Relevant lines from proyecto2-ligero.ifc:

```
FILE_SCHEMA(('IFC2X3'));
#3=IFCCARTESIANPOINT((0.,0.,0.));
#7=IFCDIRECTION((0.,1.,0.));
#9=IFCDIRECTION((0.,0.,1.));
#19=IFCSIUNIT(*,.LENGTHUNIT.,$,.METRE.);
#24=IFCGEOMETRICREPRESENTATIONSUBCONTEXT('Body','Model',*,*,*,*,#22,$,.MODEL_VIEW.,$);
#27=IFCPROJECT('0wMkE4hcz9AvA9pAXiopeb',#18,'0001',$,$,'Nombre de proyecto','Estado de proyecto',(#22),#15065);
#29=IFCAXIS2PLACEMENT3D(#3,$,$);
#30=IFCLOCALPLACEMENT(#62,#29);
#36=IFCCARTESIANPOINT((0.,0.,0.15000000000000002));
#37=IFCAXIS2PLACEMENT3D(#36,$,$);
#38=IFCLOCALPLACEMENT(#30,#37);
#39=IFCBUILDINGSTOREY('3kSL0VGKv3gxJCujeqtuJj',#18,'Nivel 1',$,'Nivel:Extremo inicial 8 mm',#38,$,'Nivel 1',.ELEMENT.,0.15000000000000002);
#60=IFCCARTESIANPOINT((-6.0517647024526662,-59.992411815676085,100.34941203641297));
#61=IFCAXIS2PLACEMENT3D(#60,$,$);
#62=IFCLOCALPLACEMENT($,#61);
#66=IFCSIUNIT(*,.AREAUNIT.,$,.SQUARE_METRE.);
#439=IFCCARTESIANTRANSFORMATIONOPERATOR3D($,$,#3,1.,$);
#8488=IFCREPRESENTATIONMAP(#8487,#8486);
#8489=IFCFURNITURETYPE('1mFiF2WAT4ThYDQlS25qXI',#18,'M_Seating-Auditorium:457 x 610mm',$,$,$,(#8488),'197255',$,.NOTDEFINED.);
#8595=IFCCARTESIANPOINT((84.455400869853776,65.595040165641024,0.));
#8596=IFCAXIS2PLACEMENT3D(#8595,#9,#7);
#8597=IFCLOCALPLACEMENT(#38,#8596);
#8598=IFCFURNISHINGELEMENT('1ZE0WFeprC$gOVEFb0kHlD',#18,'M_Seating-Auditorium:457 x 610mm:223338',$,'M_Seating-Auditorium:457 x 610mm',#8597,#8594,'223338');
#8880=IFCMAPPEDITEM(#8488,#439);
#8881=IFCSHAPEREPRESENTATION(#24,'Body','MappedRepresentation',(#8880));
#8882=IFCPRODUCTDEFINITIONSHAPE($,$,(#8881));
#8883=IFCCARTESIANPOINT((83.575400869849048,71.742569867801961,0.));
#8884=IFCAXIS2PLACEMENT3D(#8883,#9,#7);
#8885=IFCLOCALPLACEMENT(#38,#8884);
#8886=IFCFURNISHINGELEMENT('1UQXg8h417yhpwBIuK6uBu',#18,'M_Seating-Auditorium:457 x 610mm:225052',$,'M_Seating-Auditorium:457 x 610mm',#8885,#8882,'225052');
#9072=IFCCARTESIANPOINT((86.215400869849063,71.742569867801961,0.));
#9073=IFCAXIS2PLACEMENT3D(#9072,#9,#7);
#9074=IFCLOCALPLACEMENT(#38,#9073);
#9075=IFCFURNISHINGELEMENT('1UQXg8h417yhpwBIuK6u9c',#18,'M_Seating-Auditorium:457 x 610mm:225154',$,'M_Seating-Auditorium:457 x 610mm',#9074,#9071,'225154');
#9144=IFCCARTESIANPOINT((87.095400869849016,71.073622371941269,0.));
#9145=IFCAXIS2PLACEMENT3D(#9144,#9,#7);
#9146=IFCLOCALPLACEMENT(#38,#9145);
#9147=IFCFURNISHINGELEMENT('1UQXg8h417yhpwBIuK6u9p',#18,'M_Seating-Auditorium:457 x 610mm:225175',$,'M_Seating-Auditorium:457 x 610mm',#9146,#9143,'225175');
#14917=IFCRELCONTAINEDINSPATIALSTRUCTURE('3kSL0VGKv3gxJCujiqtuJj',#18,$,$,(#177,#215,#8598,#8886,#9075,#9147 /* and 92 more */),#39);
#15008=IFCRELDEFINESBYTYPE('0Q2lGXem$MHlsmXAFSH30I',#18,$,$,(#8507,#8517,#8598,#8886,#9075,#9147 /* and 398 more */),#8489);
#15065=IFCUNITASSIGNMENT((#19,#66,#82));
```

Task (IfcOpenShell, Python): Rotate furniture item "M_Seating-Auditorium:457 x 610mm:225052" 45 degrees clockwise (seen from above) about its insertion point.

```python
import ifcopenshell
import ifcopenshell.api.geometry
import ifcopenshell.util.placement

model = ifcopenshell.open("proyecto2-ligero.ifc")

item = model.by_guid("1UQXg8h417yhpwBIuK6uBu")
matrix = ifcopenshell.util.placement.get_local_placement(item.ObjectPlacement)
matrix = matrix @ ifcopenshell.util.placement.rotation(-45, "Z")
ifcopenshell.api.geometry.edit_object_placement(model, product=item, matrix=matrix, is_si=False)

print(ifcopenshell.util.placement.get_local_placement(item.ObjectPlacement).round(3) + 0.0)

model.write("proyecto2-ligero-out.ifc")
```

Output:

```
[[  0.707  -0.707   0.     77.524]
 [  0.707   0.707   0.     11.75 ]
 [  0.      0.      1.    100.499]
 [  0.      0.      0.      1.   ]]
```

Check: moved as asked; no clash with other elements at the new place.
